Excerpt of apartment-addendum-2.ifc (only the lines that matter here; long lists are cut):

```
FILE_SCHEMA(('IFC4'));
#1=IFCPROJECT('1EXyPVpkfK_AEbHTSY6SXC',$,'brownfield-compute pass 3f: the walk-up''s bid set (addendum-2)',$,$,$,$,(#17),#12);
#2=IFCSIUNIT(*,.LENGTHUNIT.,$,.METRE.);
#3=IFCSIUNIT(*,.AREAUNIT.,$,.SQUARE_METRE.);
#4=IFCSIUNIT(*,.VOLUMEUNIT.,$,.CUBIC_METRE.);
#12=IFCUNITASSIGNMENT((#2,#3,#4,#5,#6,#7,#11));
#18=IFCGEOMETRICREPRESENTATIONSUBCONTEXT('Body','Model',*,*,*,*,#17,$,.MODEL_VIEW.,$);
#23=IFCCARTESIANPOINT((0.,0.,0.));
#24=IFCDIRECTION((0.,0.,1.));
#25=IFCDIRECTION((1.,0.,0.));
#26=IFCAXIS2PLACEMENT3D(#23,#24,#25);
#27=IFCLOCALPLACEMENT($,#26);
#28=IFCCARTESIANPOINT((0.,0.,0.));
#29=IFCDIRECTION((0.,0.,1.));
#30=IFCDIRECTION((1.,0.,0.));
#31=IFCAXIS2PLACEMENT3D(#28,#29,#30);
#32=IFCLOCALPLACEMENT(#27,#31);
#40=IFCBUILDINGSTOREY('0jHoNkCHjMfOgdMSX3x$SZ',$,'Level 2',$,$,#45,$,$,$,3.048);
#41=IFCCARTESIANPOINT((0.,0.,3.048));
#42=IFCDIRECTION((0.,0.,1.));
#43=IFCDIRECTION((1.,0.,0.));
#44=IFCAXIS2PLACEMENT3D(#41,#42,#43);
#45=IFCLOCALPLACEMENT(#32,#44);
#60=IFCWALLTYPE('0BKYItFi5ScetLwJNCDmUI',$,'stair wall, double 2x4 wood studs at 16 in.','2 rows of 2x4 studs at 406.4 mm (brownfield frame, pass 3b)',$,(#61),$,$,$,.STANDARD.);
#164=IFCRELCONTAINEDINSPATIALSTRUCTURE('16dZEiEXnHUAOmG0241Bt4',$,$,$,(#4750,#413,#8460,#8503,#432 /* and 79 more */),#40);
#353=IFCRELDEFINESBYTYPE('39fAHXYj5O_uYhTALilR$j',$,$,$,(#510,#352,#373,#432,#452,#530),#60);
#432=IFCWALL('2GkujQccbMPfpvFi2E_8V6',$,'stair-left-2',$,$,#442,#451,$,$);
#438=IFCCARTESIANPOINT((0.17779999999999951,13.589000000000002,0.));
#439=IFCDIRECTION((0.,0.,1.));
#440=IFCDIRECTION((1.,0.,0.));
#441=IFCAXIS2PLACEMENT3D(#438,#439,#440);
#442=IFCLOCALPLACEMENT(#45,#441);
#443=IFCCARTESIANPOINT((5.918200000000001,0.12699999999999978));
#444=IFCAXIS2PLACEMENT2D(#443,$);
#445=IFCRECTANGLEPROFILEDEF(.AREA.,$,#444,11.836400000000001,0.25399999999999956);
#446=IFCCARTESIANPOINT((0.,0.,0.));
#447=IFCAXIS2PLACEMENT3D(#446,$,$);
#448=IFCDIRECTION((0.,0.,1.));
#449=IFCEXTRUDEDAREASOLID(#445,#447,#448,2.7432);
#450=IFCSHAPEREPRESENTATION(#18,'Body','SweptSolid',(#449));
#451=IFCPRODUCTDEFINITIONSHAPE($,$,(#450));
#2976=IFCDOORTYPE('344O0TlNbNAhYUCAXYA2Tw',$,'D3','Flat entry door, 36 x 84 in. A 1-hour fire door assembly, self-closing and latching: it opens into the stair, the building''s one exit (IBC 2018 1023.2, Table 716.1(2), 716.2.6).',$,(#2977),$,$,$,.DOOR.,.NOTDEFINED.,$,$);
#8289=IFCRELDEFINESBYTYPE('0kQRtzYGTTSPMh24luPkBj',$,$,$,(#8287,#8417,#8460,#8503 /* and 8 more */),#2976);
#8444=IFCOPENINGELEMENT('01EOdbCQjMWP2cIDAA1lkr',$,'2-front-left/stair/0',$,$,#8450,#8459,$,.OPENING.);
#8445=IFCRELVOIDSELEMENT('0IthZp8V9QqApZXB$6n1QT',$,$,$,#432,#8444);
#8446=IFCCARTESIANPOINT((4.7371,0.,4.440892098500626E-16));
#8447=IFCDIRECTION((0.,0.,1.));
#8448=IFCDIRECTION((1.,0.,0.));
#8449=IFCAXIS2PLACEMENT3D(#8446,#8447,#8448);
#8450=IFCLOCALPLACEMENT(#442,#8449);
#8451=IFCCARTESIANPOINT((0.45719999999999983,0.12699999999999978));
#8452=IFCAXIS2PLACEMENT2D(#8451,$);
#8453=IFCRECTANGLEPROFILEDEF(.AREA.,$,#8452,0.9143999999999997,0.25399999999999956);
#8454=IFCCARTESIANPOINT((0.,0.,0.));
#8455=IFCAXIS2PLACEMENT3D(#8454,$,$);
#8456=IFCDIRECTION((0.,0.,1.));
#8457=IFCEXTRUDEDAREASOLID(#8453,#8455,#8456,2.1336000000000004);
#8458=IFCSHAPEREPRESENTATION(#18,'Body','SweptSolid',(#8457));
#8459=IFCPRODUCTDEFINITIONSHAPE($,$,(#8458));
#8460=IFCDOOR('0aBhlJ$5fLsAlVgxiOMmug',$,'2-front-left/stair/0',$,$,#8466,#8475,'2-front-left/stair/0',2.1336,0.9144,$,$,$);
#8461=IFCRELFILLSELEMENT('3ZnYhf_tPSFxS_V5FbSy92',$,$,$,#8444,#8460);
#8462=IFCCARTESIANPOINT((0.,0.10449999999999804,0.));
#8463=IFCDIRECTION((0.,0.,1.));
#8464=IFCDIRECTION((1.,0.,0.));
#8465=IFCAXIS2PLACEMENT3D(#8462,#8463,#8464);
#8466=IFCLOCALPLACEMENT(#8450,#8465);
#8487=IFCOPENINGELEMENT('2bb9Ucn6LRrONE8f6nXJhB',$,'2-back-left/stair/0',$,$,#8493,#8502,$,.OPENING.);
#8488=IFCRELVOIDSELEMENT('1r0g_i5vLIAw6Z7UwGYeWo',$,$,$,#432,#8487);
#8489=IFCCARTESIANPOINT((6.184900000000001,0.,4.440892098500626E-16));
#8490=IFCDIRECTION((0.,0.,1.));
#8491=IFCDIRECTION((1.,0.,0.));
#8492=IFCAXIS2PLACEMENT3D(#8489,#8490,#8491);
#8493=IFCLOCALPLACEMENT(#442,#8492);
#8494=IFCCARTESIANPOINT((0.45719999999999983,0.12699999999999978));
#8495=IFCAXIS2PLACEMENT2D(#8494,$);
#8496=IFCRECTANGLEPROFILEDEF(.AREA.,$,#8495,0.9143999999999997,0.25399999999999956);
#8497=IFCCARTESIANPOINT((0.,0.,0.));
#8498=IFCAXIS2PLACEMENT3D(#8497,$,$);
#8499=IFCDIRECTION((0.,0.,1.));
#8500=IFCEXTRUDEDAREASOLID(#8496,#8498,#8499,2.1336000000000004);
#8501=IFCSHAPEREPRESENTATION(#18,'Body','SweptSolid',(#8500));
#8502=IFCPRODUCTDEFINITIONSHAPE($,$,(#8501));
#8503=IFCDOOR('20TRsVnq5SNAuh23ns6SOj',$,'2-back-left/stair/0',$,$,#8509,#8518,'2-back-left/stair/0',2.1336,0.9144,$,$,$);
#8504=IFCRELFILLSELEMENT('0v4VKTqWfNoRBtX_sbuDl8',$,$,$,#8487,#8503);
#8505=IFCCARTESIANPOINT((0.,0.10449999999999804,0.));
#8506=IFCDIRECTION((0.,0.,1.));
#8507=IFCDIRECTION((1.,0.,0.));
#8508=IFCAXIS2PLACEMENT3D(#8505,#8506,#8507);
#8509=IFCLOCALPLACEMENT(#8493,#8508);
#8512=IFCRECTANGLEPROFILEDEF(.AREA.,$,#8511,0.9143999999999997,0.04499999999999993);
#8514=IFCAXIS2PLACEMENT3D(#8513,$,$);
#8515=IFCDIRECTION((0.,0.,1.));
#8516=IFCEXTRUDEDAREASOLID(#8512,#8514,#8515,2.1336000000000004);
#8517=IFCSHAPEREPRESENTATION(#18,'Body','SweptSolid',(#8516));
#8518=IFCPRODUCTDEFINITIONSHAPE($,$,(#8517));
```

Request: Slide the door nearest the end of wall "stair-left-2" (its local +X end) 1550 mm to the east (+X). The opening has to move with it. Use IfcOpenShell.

```python
import ifcopenshell
import ifcopenshell.api.geometry
import ifcopenshell.util.placement

model = ifcopenshell.open("apartment-addendum-2.ifc")

door = model.by_guid("20TRsVnq5SNAuh23ns6SOj")
opening = door.FillsVoids[0].RelatingOpeningElement
wall = opening.VoidsElements[0].RelatingBuildingElement

wall_matrix = ifcopenshell.util.placement.get_local_placement(wall.ObjectPlacement)
shift = wall_matrix[:3, 0] * 1.55
before = ifcopenshell.util.placement.get_local_placement(door.ObjectPlacement)[:3, 3].copy()

# The door is placed relative to its opening, so it follows when the opening moves.
matrix = ifcopenshell.util.placement.get_local_placement(opening.ObjectPlacement)
matrix[:3, 3] += shift
ifcopenshell.api.geometry.edit_object_placement(
    model, product=opening, matrix=matrix, is_si=False, should_transform_children=True
)

after = ifcopenshell.util.placement.get_local_placement(door.ObjectPlacement)[:3, 3]
print("door moved by", (after - before).round(3) + 0.0)

model.write("apartment-addendum-2_edited.ifc")
```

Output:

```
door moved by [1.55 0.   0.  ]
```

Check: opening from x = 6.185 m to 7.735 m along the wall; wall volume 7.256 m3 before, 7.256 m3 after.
